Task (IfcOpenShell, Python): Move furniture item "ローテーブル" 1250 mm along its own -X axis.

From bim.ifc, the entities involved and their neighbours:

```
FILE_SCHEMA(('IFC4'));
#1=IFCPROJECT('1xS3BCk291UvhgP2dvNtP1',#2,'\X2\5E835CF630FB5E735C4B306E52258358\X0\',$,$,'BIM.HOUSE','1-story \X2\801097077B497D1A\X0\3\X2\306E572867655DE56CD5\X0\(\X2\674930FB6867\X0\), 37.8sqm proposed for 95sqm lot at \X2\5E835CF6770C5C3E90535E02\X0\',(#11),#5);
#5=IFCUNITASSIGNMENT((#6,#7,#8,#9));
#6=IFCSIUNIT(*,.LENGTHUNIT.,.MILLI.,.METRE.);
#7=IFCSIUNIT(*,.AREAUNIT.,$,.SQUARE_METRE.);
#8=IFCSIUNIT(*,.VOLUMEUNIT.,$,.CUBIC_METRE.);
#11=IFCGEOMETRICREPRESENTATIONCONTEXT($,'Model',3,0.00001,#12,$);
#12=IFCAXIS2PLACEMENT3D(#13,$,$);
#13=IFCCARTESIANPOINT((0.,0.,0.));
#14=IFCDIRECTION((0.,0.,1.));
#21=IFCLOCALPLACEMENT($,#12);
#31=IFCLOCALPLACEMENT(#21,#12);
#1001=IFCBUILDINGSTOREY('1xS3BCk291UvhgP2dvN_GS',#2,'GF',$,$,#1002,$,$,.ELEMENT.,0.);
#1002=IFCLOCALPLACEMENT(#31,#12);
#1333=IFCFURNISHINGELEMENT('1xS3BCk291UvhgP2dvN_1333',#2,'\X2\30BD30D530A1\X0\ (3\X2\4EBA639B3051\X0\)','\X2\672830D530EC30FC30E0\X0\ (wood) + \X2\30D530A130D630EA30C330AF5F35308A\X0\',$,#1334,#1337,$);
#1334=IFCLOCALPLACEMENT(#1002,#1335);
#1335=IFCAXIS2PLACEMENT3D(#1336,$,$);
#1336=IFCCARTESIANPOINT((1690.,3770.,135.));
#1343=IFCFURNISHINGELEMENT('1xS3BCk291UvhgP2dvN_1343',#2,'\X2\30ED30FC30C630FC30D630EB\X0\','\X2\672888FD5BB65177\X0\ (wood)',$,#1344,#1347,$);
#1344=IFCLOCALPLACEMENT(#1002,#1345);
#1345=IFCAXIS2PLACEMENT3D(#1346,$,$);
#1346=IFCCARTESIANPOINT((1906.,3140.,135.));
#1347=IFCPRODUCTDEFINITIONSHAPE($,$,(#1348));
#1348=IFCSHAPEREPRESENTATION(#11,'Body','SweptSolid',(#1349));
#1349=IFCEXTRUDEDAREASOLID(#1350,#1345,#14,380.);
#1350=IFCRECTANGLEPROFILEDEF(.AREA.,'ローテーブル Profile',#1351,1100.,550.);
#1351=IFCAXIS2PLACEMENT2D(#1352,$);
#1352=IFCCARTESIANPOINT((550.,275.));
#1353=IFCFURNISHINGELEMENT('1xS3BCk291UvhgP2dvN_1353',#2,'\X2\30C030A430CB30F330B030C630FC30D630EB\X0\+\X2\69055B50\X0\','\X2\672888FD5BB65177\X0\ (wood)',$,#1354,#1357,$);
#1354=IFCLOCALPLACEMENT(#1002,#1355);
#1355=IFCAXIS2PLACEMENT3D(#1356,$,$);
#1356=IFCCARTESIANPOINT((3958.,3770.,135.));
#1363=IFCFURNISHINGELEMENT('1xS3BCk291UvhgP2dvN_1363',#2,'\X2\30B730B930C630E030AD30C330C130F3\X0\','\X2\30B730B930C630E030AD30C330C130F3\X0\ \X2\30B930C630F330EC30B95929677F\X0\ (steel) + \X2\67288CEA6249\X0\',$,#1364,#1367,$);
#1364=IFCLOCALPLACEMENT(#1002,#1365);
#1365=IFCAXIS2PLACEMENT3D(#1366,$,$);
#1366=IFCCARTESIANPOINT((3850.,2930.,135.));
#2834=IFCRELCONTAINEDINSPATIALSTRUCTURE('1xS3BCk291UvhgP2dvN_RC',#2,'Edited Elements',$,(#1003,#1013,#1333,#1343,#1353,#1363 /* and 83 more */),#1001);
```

```python
import ifcopenshell
import ifcopenshell.api.geometry
import ifcopenshell.util.placement

model = ifcopenshell.open("bim.ifc")

item = model.by_guid("1xS3BCk291UvhgP2dvN_1343")
matrix = ifcopenshell.util.placement.get_local_placement(item.ObjectPlacement)
matrix[:3, 3] -= matrix[:3, 0] * 1250.0
ifcopenshell.api.geometry.edit_object_placement(model, product=item, matrix=matrix, is_si=False)

print(ifcopenshell.util.placement.get_local_placement(item.ObjectPlacement).round(3) + 0.0)

model.write("bim-out.ifc")
```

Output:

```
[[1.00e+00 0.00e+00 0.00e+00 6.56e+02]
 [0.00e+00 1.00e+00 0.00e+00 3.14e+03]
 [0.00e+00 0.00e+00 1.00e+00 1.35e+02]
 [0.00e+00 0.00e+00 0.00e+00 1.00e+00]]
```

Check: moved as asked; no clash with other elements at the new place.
